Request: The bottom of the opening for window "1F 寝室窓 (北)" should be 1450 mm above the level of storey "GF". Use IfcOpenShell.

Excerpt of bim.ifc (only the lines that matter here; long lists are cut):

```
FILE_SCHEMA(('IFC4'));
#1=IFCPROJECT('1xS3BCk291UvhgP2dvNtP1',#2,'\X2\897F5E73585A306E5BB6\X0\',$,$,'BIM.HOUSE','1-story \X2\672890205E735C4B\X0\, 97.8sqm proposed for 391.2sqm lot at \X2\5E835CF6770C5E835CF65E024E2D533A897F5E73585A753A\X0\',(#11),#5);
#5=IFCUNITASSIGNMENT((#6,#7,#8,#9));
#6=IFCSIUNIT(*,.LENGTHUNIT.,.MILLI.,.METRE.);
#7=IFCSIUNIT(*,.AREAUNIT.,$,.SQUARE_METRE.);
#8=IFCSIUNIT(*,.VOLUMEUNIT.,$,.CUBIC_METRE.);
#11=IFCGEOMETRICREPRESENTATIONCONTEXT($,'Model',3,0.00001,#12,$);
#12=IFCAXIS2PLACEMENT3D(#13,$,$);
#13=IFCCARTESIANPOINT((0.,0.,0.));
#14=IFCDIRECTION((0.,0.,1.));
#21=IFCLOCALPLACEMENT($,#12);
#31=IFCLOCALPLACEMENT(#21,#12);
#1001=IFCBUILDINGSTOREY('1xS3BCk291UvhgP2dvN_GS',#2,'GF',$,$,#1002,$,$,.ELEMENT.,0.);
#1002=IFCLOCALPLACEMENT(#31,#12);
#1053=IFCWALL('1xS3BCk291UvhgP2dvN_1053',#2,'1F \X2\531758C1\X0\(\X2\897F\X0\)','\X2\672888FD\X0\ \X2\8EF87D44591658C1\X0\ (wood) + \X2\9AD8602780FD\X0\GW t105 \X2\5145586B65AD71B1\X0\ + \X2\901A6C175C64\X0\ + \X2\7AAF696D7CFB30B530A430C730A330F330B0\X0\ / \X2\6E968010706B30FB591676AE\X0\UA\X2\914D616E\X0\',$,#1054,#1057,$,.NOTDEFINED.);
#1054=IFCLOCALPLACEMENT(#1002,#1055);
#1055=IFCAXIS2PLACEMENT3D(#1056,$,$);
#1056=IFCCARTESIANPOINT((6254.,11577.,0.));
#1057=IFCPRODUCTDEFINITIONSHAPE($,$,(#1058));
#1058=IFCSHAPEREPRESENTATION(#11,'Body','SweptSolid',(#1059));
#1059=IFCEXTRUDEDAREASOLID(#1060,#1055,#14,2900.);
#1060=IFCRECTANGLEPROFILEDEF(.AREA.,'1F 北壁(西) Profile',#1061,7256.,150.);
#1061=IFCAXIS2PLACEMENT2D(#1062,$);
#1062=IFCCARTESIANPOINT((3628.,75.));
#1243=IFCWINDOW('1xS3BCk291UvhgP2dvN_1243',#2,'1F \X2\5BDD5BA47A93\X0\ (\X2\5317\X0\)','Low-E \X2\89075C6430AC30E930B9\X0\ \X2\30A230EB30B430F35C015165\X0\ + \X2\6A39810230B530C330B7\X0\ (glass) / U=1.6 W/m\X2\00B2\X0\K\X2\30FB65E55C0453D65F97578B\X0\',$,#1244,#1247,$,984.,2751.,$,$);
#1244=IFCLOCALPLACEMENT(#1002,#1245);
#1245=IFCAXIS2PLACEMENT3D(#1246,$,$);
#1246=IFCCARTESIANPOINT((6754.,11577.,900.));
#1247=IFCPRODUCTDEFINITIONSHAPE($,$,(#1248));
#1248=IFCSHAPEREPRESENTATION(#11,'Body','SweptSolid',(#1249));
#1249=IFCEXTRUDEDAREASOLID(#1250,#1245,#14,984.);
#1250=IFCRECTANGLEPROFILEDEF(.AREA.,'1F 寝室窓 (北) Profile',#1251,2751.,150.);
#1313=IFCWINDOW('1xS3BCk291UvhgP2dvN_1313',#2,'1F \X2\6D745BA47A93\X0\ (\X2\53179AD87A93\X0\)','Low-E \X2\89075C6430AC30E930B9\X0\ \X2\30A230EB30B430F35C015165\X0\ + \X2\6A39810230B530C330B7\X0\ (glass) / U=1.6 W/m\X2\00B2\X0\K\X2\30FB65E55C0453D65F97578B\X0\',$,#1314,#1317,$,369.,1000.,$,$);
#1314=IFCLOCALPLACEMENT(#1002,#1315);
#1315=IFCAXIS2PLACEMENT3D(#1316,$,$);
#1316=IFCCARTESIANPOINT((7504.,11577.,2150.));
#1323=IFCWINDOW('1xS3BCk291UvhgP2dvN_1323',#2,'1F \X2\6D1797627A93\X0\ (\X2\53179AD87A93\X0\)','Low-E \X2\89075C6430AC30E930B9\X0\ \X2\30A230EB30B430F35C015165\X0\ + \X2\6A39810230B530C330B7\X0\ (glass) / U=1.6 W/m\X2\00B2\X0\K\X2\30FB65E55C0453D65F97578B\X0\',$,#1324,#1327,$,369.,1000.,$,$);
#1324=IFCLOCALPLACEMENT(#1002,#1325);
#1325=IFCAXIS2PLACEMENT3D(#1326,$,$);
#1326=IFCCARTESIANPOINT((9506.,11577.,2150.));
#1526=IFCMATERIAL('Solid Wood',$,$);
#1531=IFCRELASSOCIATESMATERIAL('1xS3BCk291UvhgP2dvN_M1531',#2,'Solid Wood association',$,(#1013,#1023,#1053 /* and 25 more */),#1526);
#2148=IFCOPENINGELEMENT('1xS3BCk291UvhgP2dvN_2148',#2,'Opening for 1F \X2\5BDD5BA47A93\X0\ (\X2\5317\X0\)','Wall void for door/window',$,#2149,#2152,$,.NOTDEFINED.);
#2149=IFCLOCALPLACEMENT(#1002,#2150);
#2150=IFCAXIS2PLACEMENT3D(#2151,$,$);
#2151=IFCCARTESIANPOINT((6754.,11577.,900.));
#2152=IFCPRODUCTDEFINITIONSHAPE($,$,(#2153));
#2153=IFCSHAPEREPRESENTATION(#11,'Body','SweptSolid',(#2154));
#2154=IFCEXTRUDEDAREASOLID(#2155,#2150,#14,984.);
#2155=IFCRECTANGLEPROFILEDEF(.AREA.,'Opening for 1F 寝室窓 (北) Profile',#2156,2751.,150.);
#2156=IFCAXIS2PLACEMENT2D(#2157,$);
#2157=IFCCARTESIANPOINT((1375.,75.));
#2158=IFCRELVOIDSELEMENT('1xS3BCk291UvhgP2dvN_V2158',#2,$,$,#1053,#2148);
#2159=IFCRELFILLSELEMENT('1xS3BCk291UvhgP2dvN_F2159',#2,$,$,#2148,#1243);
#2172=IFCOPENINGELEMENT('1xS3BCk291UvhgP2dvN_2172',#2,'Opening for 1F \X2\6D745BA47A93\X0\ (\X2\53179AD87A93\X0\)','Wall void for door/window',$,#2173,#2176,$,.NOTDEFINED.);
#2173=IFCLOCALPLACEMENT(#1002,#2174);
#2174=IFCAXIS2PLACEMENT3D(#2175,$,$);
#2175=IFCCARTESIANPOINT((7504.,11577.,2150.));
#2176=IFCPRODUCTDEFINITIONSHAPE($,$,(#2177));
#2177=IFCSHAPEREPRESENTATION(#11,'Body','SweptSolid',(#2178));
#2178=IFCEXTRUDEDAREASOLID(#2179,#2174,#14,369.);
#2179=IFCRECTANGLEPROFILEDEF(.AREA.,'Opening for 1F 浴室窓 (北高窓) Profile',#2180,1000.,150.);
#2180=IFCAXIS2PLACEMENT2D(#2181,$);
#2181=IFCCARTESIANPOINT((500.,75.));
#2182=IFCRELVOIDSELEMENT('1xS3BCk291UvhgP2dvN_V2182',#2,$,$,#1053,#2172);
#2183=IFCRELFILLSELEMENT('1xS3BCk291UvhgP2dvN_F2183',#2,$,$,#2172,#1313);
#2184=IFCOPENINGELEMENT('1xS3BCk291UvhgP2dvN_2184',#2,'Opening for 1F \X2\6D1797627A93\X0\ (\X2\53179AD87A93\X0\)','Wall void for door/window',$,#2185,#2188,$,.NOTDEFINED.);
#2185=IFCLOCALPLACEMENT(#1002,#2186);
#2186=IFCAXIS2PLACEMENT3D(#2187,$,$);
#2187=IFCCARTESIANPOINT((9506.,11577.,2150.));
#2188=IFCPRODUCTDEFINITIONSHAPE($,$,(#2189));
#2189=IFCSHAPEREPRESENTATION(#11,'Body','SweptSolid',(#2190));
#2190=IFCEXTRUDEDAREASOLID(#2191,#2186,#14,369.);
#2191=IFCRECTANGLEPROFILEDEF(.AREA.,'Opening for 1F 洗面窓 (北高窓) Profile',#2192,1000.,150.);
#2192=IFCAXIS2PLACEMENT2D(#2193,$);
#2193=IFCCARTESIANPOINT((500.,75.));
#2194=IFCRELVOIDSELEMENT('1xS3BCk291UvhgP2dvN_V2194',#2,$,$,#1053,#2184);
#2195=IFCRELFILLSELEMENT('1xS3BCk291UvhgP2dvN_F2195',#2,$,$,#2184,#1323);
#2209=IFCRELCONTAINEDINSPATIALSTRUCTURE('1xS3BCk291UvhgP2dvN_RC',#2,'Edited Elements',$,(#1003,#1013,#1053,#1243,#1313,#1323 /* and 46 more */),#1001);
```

```python
import numpy as np
import ifcopenshell
import ifcopenshell.api.geometry
import ifcopenshell.geom
import ifcopenshell.util.element
import ifcopenshell.util.placement
import ifcopenshell.util.shape
import ifcopenshell.util.unit

model = ifcopenshell.open("bim.ifc")
unit_scale = ifcopenshell.util.unit.calculate_unit_scale(model)

window = model.by_id(1243)
opening = window.FillsVoids[0].RelatingOpeningElement
storey = ifcopenshell.util.element.get_container(window, ifc_class="IfcBuildingStorey")
level = ifcopenshell.util.placement.get_local_placement(storey.ObjectPlacement)[2, 3]

# The opening's origin need not be at the sill, so measure its lowest point.
shape = ifcopenshell.geom.create_shape(ifcopenshell.geom.settings(), opening)
bottom = ifcopenshell.util.shape.get_shape_bottom_elevation(shape, shape.geometry) / unit_scale
dz = level + 1.45 / unit_scale - bottom

shift = np.array([0.0, 0.0, dz])
# The window is not placed relative to its opening, so move both.
for product in (opening, window):
    matrix = ifcopenshell.util.placement.get_local_placement(product.ObjectPlacement)
    matrix[:3, 3] += shift
    ifcopenshell.api.geometry.edit_object_placement(model, product=product, matrix=matrix, is_si=False)

print(f"moved by {dz * unit_scale:+.3f} m")

model.write("bim_v2.ifc")
```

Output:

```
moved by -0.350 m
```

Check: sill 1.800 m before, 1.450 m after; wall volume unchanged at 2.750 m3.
